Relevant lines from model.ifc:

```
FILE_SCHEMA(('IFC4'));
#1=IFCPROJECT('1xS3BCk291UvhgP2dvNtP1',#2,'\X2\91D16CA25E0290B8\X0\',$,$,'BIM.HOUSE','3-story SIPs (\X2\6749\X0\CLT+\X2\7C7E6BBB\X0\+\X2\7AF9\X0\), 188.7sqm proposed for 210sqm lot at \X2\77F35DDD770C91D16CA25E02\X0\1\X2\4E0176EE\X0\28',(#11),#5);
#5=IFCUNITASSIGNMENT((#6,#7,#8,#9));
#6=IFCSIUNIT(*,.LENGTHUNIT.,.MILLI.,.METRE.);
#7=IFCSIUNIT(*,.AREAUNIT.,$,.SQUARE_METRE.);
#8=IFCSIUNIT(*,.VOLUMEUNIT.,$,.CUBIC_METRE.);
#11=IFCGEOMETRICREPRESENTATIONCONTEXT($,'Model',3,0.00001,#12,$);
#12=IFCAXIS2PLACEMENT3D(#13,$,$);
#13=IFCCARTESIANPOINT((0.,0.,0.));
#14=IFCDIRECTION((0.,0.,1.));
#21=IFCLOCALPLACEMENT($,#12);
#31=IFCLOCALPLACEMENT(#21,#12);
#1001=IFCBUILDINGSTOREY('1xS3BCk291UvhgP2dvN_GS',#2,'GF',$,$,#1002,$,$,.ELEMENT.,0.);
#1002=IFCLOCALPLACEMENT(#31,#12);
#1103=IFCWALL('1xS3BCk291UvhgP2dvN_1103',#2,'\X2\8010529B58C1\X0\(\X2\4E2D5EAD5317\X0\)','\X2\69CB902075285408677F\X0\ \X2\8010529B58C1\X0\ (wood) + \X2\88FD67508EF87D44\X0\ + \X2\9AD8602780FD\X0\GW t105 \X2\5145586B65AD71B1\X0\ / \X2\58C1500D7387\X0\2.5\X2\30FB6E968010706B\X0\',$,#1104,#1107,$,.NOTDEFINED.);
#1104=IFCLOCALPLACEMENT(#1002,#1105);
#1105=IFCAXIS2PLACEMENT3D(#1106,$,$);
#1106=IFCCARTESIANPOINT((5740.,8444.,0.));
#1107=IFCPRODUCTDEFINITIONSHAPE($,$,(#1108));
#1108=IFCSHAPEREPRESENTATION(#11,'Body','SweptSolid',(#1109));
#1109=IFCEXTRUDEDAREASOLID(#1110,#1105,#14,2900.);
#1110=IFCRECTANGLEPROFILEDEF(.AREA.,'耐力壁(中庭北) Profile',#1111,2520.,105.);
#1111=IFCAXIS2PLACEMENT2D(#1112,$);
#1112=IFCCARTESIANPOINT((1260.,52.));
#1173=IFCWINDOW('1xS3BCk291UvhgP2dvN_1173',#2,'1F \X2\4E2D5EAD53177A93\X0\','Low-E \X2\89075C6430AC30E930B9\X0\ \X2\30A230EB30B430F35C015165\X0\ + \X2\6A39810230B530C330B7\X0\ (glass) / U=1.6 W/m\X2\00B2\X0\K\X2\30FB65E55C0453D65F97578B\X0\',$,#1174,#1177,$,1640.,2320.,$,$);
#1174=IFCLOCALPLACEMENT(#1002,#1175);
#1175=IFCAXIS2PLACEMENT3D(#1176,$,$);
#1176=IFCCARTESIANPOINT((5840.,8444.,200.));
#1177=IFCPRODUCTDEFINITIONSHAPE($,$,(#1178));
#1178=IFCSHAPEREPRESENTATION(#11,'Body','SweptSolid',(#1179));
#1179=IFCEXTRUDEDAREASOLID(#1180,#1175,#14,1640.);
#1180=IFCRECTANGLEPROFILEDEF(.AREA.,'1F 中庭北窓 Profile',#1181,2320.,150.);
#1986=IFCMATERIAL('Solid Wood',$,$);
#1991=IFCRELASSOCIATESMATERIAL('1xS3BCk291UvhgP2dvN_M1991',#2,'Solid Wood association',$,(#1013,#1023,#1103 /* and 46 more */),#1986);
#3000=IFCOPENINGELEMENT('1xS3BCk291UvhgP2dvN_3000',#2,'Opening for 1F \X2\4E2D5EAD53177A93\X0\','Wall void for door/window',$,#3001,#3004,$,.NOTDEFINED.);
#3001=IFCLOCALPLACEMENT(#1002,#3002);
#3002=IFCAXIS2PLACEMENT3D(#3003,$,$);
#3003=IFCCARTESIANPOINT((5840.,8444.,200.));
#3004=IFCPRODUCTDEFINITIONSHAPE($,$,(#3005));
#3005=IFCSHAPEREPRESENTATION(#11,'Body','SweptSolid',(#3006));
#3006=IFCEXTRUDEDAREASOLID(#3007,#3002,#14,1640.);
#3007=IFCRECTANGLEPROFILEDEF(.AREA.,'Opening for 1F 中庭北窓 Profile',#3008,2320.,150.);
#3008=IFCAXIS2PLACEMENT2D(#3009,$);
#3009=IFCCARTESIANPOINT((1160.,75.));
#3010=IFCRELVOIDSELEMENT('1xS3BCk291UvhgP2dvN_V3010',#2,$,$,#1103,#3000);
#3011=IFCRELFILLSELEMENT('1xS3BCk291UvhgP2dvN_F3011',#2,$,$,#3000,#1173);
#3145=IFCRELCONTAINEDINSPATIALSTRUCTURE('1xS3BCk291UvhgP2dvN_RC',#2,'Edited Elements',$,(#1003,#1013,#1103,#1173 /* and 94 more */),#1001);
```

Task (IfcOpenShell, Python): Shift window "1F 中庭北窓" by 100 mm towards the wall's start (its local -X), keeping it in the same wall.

```python
import ifcopenshell
import ifcopenshell.api.geometry
import ifcopenshell.util.placement
import ifcopenshell.util.unit

model = ifcopenshell.open("model.ifc")
unit_scale = ifcopenshell.util.unit.calculate_unit_scale(model)

window = model.by_id(1173)
opening = window.FillsVoids[0].RelatingOpeningElement
wall = opening.VoidsElements[0].RelatingBuildingElement

wall_matrix = ifcopenshell.util.placement.get_local_placement(wall.ObjectPlacement)
shift = wall_matrix[:3, 0] * -0.1 / unit_scale
before = ifcopenshell.util.placement.get_local_placement(window.ObjectPlacement)[:3, 3].copy()

# The window is not placed relative to its opening, so move both.
for product in (opening, window):
    matrix = ifcopenshell.util.placement.get_local_placement(product.ObjectPlacement)
    matrix[:3, 3] += shift
    ifcopenshell.api.geometry.edit_object_placement(model, product=product, matrix=matrix, is_si=False)

after = ifcopenshell.util.placement.get_local_placement(window.ObjectPlacement)[:3, 3]
print("window moved by", (after - before).round(3) + 0.0)

model.write("model-out.ifc")
```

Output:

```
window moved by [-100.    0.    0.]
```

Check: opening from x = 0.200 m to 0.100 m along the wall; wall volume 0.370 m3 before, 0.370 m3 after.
